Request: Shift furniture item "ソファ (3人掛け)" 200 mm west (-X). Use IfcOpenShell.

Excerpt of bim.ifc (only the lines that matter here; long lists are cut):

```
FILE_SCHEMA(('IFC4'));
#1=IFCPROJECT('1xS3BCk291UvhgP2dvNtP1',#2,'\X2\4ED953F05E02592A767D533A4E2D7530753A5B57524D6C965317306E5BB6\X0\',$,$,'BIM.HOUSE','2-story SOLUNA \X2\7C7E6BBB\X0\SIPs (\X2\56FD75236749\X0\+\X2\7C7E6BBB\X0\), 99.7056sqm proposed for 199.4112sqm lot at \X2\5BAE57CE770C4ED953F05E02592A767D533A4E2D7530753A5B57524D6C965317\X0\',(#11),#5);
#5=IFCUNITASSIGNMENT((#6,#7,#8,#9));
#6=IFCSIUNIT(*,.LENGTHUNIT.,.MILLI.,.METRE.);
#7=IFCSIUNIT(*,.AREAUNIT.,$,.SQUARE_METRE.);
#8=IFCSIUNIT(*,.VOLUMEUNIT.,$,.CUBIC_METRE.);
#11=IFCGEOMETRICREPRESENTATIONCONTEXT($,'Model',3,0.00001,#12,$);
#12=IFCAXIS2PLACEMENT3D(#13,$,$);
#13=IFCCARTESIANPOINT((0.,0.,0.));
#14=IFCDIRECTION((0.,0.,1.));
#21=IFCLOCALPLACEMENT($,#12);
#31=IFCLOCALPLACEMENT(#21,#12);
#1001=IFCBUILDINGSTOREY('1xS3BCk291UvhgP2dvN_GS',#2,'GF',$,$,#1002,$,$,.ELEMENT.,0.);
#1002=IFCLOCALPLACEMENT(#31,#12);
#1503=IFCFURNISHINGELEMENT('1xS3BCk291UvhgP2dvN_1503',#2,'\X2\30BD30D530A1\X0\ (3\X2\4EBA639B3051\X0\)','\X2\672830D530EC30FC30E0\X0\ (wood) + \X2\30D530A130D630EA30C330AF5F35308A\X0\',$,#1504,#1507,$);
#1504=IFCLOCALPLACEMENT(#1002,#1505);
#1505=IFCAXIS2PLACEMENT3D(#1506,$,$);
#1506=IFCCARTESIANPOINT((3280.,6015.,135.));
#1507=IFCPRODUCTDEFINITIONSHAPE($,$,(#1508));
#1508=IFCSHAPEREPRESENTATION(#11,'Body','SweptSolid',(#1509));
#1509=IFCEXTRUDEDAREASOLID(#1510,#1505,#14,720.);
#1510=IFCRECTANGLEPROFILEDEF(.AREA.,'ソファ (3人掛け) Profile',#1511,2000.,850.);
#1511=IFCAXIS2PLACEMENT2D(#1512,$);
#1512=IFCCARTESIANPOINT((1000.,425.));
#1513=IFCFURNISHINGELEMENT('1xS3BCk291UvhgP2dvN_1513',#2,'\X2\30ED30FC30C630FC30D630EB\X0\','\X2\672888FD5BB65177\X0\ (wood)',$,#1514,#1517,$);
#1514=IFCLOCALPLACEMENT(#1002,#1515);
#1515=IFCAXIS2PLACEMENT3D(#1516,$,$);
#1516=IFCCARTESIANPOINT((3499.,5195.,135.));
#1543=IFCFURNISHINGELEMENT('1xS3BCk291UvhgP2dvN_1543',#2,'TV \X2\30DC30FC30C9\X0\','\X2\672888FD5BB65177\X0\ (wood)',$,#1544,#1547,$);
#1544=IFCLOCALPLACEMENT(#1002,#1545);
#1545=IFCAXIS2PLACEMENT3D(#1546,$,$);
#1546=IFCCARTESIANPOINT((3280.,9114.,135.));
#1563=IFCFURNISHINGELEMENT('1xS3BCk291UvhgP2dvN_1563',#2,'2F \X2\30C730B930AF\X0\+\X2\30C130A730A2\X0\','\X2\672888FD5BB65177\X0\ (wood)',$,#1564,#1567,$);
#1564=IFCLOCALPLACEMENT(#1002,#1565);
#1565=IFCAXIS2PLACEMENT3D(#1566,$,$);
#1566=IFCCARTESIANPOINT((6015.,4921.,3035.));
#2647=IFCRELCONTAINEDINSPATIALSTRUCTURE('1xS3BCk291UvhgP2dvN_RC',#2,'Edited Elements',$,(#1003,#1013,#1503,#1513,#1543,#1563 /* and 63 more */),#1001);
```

```python
import ifcopenshell
import ifcopenshell.api.geometry
import ifcopenshell.util.placement
import ifcopenshell.util.unit

model = ifcopenshell.open("bim.ifc")
unit_scale = ifcopenshell.util.unit.calculate_unit_scale(model)

item = model.by_id(1503)
matrix = ifcopenshell.util.placement.get_local_placement(item.ObjectPlacement)
matrix[0, 3] -= 0.2 / unit_scale
ifcopenshell.api.geometry.edit_object_placement(model, product=item, matrix=matrix, is_si=False)

print(ifcopenshell.util.placement.get_local_placement(item.ObjectPlacement).round(3) + 0.0)

model.write("bim-out.ifc")
```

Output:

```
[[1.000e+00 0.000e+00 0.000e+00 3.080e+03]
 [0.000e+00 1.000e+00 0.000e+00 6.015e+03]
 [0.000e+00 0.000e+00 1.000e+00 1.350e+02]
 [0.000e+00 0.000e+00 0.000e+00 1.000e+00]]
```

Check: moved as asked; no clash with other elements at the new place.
